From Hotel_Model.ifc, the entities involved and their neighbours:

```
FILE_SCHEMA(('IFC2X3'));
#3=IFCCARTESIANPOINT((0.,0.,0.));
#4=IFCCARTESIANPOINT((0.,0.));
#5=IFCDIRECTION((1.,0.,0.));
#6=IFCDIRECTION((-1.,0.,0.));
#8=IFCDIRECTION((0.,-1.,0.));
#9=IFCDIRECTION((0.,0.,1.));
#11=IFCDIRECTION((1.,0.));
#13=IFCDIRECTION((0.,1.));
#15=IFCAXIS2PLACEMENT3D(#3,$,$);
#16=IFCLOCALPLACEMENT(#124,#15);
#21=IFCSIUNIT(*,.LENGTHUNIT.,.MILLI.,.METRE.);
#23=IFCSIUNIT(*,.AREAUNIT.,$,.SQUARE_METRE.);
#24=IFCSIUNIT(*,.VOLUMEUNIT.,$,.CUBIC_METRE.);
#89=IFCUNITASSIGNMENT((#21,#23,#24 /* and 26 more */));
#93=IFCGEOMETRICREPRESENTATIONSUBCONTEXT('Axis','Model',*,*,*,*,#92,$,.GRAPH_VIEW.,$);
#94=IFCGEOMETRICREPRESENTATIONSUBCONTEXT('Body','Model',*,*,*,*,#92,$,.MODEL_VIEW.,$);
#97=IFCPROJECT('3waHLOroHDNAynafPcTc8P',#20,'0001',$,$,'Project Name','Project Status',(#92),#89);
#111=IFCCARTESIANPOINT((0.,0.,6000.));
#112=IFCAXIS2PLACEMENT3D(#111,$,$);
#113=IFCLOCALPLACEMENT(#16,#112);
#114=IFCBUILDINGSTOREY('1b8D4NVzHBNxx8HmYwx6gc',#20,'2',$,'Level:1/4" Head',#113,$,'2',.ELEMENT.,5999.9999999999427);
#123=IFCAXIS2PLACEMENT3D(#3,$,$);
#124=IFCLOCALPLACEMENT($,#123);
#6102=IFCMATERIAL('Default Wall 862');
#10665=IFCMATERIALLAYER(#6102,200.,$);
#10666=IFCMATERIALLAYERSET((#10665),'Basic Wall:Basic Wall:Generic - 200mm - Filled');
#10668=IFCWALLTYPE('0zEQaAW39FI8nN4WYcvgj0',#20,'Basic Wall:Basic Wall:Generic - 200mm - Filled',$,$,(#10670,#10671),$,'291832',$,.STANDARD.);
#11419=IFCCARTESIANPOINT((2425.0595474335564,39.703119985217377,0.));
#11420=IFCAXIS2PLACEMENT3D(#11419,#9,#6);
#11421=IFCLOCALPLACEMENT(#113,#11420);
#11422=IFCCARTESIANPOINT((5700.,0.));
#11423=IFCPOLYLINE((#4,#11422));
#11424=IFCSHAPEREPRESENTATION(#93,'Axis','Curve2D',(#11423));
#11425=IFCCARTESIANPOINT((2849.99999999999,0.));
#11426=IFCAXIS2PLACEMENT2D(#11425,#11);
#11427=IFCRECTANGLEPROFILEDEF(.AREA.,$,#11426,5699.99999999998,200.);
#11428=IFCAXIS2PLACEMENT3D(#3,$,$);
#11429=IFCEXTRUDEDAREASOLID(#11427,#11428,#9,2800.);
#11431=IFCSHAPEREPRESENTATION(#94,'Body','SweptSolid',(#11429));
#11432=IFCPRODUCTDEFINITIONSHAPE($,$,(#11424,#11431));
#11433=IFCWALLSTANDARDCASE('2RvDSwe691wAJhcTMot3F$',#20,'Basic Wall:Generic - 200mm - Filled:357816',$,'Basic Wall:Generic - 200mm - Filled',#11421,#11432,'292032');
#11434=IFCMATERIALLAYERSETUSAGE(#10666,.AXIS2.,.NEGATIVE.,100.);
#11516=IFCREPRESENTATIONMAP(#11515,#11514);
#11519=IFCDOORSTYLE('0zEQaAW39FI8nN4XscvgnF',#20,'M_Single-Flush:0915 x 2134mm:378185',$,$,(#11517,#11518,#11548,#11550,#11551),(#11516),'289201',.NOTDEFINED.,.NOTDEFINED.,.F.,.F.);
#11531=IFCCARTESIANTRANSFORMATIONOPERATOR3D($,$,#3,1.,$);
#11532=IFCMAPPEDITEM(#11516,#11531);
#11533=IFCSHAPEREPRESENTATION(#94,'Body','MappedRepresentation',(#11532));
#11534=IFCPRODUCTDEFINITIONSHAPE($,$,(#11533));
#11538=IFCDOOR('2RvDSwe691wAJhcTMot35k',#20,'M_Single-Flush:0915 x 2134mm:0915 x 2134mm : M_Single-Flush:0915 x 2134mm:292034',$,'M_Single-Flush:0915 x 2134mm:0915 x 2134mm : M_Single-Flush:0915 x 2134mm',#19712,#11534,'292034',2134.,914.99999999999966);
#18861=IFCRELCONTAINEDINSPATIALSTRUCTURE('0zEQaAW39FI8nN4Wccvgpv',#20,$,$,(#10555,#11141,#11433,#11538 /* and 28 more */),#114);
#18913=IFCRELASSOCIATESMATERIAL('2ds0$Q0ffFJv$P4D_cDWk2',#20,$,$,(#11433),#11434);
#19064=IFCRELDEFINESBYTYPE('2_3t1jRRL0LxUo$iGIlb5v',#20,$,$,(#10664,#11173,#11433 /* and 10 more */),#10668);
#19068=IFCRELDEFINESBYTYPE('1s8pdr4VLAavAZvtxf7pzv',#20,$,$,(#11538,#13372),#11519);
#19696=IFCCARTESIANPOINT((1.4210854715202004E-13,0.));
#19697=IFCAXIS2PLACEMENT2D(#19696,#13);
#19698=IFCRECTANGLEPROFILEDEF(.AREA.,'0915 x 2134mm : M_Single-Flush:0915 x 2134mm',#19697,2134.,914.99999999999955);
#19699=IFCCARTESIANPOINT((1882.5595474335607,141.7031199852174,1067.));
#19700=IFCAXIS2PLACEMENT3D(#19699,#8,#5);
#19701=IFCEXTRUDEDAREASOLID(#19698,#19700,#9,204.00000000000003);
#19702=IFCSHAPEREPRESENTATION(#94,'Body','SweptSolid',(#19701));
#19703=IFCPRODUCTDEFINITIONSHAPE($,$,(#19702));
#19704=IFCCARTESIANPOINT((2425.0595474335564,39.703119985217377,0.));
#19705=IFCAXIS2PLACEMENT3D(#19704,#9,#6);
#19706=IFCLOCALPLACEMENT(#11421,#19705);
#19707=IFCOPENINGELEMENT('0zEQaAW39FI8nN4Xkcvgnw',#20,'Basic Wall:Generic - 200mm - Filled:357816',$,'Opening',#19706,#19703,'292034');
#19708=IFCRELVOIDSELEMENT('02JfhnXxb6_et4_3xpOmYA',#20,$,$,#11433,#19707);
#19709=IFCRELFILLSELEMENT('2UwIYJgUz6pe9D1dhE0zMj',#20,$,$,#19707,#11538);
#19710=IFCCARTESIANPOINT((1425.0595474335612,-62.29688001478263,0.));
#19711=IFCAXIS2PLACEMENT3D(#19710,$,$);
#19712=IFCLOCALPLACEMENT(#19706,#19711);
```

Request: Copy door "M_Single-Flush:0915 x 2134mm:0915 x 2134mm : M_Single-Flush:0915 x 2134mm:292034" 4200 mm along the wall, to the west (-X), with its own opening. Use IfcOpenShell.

```python
import ifcopenshell
import ifcopenshell.api.feature
import ifcopenshell.api.geometry
import ifcopenshell.api.root
import ifcopenshell.geom
import ifcopenshell.util.element
import ifcopenshell.util.placement
import ifcopenshell.util.shape
import ifcopenshell.util.unit

model = ifcopenshell.open("Hotel_Model.ifc")
unit_scale = ifcopenshell.util.unit.calculate_unit_scale(model)
settings = ifcopenshell.geom.settings()


def volume(element):
    """Net volume in cubic metres, openings subtracted."""
    shape = ifcopenshell.geom.create_shape(settings, element)
    return ifcopenshell.util.shape.get_volume(shape.geometry)


def reuse_history(source, copy):
    """copy_class also copies each property set's owner history, people and application; keep the originals."""
    for rel in copy.IsDefinedBy:
        if rel.is_a("IfcRelDefinesByProperties") and (history := rel.RelatingPropertyDefinition.OwnerHistory):
            rel.RelatingPropertyDefinition.OwnerHistory = source.OwnerHistory
            ifcopenshell.util.element.remove_deep2(model, history)


door = model.by_guid("2RvDSwe691wAJhcTMot35k")
opening = door.FillsVoids[0].RelatingOpeningElement
wall = opening.VoidsElements[0].RelatingBuildingElement
before = volume(wall)
shift = ifcopenshell.util.placement.get_local_placement(wall.ObjectPlacement)[:3, 0] * 4.2 / unit_scale

# copy_class copies the void relationship, type, container and properties, but no geometry.
new_opening = ifcopenshell.api.root.copy_class(model, product=opening)
new_opening.Representation = ifcopenshell.util.element.copy_deep(
    model, opening.Representation, exclude=["IfcGeometricRepresentationContext", "IfcRepresentationMap"]
)
new_opening.Name = "Basic Wall:Generic - 200mm - Filled"
new_opening.Tag = None
new_door = ifcopenshell.api.root.copy_class(model, product=door)
new_door.Representation = ifcopenshell.util.element.copy_deep(
    model, door.Representation, exclude=["IfcGeometricRepresentationContext", "IfcRepresentationMap"]
)
new_door.Name = "M_Single-Flush:0915 x 2134mm:0915 x 2134mm : M_Single-Flush:0915 x 2134mm"
new_door.Tag = None
reuse_history(door, new_door)
fills = ifcopenshell.api.feature.add_filling(model, opening=new_opening, element=new_door)
fills.OwnerHistory = new_door.OwnerHistory  # required in IFC2X3

for old, new in ((opening, new_opening), (door, new_door)):
    matrix = ifcopenshell.util.placement.get_local_placement(old.ObjectPlacement)
    matrix[:3, 3] += shift
    ifcopenshell.api.geometry.edit_object_placement(model, product=new, matrix=matrix, is_si=False)

after = volume(wall)

print(f"wall volume {before:.3f} -> {after:.3f} m3")

model.write("Hotel_Model_updated.ifc")
```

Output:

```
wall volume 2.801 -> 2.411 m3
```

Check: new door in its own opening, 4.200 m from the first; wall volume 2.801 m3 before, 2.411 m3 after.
